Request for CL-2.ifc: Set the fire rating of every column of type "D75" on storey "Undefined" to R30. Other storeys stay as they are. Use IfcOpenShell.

First a look at what the model holds.

```python
import ifcopenshell
import ifcopenshell.util.element

model = ifcopenshell.open("CL-2.ifc")
print(model.schema)
storey = next(s for s in model.by_type("IfcBuildingStorey") if s.Name == "Undefined")
columns = [e for e in ifcopenshell.util.element.get_decomposition(storey) if e.is_a("IfcColumn")]
seen = {}
for e in columns:
    element_type = ifcopenshell.util.element.get_type(e)
    key = (element_type.Name if element_type != e and element_type else None, ifcopenshell.util.element.get_pset(e, "Pset_ColumnCommon", "FireRating"))
    seen[key] = seen.get(key, 0) + 1
for (name, value), count in sorted(seen.items(), key=str):
    print(count, "x", name, "|", value)
```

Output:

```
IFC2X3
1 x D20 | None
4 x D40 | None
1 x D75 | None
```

```python
import ifcopenshell
import ifcopenshell.api.pset
import ifcopenshell.util.element

model = ifcopenshell.open("CL-2.ifc")

storey = next(s for s in model.by_type("IfcBuildingStorey") if s.Name == "Undefined")
columns = [e for e in ifcopenshell.util.element.get_decomposition(storey) if e.is_a("IfcColumn")]

count = 0
for e in columns:
    element_type = ifcopenshell.util.element.get_type(e)
    if element_type in (None, e) or element_type.Name != "D75":
        continue
    # add_pset returns the element's existing set when there is one.
    pset = ifcopenshell.api.pset.add_pset(model, product=e, name="Pset_ColumnCommon")
    ifcopenshell.api.pset.edit_pset(model, pset=pset, properties={"FireRating": "R30"})
    count += 1

print(count, "columns updated")

model.write("CL-2_v2.ifc")
```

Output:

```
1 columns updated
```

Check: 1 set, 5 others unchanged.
